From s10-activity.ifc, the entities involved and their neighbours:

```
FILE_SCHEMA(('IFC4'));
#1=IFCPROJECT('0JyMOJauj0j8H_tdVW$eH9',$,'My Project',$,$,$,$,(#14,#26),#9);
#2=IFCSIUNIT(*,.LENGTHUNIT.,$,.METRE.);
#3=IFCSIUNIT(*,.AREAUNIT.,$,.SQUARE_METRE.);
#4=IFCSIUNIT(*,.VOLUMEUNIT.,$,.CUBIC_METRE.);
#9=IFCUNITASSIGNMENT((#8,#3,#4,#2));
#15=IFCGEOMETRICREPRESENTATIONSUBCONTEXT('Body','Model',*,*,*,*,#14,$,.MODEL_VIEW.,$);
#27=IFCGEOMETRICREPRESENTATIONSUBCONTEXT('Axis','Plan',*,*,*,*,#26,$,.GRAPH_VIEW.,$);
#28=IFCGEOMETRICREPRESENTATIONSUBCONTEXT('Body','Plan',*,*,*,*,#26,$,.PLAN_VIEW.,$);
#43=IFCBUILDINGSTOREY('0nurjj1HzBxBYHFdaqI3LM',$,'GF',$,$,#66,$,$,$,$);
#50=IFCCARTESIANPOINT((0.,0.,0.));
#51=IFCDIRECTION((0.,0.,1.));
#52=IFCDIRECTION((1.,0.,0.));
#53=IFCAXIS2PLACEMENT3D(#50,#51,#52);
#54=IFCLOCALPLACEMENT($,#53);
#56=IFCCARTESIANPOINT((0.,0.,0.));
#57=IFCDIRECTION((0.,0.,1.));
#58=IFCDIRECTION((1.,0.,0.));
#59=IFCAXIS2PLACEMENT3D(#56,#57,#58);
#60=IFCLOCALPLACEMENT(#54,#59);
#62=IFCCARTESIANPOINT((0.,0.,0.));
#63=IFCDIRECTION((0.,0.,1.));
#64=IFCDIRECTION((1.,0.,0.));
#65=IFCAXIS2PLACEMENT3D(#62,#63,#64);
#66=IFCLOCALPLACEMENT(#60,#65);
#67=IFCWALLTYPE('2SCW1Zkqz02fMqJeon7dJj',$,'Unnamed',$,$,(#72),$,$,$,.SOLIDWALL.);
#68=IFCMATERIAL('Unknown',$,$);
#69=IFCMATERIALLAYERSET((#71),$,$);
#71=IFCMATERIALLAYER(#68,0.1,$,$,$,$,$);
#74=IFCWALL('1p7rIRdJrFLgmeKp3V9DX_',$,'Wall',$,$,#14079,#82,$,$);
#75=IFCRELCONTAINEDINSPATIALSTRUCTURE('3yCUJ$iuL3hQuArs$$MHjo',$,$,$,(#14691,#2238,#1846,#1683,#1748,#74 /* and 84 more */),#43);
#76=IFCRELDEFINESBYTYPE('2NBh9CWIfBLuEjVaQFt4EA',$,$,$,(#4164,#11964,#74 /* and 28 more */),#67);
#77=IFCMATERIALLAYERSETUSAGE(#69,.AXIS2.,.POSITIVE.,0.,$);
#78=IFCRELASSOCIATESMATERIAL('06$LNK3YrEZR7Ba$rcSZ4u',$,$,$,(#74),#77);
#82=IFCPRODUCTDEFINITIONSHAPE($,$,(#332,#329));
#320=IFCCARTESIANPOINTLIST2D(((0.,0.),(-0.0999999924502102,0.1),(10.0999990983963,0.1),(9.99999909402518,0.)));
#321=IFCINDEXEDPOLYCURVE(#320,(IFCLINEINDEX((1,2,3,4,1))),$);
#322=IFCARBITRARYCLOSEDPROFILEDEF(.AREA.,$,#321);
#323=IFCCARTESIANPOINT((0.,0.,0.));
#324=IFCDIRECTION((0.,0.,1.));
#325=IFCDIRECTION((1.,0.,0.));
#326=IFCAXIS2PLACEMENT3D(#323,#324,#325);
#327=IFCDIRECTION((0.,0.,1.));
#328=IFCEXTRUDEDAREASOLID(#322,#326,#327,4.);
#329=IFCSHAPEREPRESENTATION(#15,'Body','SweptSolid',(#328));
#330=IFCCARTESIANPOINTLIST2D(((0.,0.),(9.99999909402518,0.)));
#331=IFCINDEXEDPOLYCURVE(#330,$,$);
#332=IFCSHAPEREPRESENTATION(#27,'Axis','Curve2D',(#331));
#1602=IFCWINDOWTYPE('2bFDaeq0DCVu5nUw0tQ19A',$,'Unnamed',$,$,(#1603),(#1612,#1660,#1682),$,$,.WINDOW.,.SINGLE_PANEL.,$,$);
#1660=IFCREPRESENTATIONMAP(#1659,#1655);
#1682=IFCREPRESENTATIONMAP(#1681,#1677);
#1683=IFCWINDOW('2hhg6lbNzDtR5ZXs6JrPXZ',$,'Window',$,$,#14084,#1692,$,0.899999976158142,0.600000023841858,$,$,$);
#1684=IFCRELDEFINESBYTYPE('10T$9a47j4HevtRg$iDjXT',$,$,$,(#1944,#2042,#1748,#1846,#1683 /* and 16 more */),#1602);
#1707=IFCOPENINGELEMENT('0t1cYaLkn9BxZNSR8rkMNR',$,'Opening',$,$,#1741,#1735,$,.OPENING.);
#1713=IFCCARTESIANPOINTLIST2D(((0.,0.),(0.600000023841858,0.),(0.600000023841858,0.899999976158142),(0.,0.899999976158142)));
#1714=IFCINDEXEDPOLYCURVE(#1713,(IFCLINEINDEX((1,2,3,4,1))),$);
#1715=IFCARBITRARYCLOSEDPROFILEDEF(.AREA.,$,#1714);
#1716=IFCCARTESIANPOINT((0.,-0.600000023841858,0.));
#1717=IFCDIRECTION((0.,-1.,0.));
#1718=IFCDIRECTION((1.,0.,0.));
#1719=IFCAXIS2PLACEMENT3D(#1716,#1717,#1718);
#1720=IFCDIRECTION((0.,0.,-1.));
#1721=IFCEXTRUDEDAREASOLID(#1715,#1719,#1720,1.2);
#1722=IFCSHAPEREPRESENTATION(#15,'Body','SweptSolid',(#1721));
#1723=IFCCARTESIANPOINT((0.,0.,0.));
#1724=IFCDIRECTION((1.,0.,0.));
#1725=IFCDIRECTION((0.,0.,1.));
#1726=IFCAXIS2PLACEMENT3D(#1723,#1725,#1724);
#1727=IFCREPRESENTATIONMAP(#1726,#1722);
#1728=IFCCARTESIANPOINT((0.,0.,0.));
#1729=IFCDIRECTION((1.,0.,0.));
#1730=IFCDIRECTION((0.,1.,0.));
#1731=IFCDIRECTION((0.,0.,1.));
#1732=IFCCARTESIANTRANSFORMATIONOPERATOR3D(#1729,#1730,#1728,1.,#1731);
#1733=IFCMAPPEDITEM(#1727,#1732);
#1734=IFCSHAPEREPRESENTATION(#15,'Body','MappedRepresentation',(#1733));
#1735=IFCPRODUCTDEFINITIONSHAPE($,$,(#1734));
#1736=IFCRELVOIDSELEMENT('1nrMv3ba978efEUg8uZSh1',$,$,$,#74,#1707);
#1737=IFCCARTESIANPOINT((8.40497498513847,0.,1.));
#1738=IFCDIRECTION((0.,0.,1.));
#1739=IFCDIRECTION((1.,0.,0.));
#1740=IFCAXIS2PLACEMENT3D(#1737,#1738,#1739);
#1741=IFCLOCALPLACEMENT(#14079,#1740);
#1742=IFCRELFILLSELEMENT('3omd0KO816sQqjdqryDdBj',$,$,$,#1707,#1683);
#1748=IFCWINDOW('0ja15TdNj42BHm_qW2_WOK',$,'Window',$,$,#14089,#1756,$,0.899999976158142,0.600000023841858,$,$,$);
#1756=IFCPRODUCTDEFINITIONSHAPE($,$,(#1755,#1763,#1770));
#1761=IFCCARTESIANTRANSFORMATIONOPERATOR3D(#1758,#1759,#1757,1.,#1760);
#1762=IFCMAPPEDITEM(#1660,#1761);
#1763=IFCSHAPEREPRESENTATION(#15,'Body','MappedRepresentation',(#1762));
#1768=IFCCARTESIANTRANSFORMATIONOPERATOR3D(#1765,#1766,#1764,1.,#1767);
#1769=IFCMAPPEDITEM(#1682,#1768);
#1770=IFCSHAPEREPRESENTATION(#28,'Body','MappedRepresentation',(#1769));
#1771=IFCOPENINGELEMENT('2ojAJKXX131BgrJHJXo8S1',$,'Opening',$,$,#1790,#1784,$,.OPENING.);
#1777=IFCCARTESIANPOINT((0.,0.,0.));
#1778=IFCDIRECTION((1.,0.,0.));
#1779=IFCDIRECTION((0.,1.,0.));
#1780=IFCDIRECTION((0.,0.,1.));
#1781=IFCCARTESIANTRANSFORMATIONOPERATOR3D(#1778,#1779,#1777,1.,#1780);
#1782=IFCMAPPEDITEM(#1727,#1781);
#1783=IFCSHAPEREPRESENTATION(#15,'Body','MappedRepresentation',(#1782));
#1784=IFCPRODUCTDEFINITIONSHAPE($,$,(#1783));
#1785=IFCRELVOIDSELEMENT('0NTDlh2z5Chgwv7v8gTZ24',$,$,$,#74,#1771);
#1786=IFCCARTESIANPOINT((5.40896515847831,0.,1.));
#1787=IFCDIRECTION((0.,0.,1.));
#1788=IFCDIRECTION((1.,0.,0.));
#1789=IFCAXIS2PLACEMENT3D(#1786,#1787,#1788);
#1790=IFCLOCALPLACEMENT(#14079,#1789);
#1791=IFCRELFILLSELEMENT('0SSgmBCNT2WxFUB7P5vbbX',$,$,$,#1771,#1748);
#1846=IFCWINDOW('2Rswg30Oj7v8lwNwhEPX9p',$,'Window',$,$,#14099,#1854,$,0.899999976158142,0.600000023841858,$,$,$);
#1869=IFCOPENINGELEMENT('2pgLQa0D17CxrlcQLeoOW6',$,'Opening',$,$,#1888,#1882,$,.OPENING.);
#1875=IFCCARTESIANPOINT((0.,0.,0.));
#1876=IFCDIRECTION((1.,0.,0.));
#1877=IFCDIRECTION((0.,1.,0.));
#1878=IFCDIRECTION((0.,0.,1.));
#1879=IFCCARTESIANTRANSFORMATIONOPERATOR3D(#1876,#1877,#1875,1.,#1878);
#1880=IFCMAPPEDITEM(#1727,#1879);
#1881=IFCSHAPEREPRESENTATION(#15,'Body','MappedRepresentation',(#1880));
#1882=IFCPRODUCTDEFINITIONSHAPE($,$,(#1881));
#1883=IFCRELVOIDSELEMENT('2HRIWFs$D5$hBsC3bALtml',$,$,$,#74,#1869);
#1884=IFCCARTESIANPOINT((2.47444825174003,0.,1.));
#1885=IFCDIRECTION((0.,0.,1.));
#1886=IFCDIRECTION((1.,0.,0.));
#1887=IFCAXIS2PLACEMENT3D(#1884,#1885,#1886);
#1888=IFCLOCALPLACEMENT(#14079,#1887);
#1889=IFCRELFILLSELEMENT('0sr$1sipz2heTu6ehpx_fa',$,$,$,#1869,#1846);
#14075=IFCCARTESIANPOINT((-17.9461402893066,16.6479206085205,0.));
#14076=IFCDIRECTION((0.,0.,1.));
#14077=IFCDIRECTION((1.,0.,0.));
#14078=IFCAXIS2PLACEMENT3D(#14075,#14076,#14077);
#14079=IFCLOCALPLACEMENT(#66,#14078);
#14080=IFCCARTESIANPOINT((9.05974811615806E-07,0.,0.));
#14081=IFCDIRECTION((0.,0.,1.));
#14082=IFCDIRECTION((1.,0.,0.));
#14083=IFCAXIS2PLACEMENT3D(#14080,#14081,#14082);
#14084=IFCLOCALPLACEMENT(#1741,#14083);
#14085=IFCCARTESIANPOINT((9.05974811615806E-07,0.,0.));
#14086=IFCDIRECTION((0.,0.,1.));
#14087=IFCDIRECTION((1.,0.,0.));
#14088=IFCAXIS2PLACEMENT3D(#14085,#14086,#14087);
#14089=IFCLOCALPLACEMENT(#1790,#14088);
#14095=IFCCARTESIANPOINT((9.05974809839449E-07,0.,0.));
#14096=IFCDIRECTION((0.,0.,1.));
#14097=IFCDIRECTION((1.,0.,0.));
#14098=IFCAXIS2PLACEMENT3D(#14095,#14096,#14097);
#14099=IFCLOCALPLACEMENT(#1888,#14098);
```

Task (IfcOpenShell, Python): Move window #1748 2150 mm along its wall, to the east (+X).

```python
import ifcopenshell
import ifcopenshell.api.geometry
import ifcopenshell.util.placement
import ifcopenshell.util.unit

model = ifcopenshell.open("s10-activity.ifc")
unit_scale = ifcopenshell.util.unit.calculate_unit_scale(model)

window = model.by_guid("0ja15TdNj42BHm_qW2_WOK")
opening = window.FillsVoids[0].RelatingOpeningElement
wall = opening.VoidsElements[0].RelatingBuildingElement

wall_matrix = ifcopenshell.util.placement.get_local_placement(wall.ObjectPlacement)
shift = wall_matrix[:3, 0] * 2.15 / unit_scale
before = ifcopenshell.util.placement.get_local_placement(window.ObjectPlacement)[:3, 3].copy()

# The window is placed relative to its opening, so it follows when the opening moves.
matrix = ifcopenshell.util.placement.get_local_placement(opening.ObjectPlacement)
matrix[:3, 3] += shift
ifcopenshell.api.geometry.edit_object_placement(
    model, product=opening, matrix=matrix, is_si=False, should_transform_children=True
)

after = ifcopenshell.util.placement.get_local_placement(window.ObjectPlacement)[:3, 3]
print("window moved by", (after - before).round(3) + 0.0)

model.write("s10-activity_edited.ifc")
```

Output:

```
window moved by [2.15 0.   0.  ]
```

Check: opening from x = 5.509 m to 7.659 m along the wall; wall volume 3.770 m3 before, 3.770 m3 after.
